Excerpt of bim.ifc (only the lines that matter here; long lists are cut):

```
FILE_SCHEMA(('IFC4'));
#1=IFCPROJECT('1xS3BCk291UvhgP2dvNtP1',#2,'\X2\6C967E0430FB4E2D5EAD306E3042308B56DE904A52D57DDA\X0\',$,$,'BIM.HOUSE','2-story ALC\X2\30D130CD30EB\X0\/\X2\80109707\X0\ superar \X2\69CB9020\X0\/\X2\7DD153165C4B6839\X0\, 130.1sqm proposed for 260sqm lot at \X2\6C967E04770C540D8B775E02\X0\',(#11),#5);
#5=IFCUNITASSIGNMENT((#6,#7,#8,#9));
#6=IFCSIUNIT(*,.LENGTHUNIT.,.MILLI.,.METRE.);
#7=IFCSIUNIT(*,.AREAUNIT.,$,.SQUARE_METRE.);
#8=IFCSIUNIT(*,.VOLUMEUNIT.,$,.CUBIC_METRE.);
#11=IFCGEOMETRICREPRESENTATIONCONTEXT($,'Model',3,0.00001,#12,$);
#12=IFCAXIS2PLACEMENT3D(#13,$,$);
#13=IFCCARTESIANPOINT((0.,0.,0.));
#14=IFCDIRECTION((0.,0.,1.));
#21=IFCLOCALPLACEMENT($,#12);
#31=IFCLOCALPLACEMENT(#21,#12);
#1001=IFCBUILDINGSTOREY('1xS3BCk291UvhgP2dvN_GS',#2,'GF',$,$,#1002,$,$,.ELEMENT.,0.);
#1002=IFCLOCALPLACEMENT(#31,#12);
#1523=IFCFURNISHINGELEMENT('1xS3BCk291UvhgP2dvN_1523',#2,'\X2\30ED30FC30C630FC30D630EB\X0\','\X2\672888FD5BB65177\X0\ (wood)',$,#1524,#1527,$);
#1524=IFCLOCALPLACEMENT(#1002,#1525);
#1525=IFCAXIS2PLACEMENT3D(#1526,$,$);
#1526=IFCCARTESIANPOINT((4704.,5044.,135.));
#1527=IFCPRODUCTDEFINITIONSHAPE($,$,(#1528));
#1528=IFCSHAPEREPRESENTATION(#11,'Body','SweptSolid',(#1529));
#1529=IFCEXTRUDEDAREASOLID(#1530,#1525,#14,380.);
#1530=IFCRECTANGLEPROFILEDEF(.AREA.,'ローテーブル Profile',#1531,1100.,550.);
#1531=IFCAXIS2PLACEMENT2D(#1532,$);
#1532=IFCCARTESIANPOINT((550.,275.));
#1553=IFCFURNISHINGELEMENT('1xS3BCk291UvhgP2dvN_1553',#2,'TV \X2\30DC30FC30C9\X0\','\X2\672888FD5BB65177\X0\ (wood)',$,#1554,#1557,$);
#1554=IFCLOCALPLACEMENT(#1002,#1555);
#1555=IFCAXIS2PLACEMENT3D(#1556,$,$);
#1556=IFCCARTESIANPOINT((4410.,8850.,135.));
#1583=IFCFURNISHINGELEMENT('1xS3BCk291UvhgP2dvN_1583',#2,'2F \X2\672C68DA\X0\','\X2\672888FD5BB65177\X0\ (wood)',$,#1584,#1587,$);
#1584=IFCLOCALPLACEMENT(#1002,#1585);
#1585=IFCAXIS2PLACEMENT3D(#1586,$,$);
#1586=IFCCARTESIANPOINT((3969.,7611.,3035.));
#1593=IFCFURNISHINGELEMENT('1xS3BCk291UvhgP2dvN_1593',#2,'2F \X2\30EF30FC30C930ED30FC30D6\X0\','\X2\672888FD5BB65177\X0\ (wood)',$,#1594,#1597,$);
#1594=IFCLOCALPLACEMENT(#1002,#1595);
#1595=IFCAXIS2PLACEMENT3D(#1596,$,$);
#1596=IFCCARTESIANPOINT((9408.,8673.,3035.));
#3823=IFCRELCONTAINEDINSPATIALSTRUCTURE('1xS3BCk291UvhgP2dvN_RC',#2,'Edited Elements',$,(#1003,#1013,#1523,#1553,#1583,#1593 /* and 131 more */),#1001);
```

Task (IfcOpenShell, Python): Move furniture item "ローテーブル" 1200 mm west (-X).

```python
import ifcopenshell
import ifcopenshell.api.geometry
import ifcopenshell.util.placement
import ifcopenshell.util.unit

model = ifcopenshell.open("bim.ifc")
unit_scale = ifcopenshell.util.unit.calculate_unit_scale(model)

item = model.by_guid("1xS3BCk291UvhgP2dvN_1523")
matrix = ifcopenshell.util.placement.get_local_placement(item.ObjectPlacement)
matrix[0, 3] -= 1.2 / unit_scale
ifcopenshell.api.geometry.edit_object_placement(model, product=item, matrix=matrix, is_si=False)

print(ifcopenshell.util.placement.get_local_placement(item.ObjectPlacement).round(3) + 0.0)

model.write("bim_rev.ifc")
```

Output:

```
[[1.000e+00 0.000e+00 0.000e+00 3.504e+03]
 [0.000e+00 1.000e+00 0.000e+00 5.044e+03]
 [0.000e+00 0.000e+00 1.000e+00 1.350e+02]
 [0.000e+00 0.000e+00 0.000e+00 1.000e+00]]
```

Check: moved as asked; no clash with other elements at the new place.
